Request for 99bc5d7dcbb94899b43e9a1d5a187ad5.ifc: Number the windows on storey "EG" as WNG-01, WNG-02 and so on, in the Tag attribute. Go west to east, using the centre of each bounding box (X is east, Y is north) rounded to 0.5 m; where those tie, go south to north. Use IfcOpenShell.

First a look at what the model holds.

```python
import ifcopenshell
import ifcopenshell.util.element
import ifcopenshell.util.placement

model = ifcopenshell.open("99bc5d7dcbb94899b43e9a1d5a187ad5.ifc")
print(model.schema)
storey = next(s for s in model.by_type("IfcBuildingStorey") if s.Name == "EG")
windows = [e for e in ifcopenshell.util.element.get_decomposition(storey) if e.is_a("IfcWindow")]
for e in sorted(windows, key=lambda e: e.id()):
    origin = ifcopenshell.util.placement.get_local_placement(e.ObjectPlacement)[:3, 3]
    print(e.id(), e.Tag, e.Name, origin.round(2) + 0.0, sep=" | ")
```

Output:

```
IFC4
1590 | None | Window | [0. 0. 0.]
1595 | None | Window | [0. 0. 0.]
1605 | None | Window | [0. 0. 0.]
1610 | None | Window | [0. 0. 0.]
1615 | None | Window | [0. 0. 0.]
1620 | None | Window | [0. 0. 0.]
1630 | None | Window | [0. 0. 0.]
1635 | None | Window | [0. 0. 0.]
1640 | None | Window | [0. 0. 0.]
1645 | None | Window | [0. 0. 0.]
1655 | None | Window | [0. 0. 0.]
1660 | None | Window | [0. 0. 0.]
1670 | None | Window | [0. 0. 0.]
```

```python
import ifcopenshell
import ifcopenshell.geom
import ifcopenshell.util.element
import ifcopenshell.util.shape

model = ifcopenshell.open("99bc5d7dcbb94899b43e9a1d5a187ad5.ifc")
settings = ifcopenshell.geom.settings()
settings.set("use-world-coords", True)


def centre(element):
    shape = ifcopenshell.geom.create_shape(settings, element)
    return ifcopenshell.util.shape.get_bbox_centroid(shape.geometry)


storey = next(s for s in model.by_type("IfcBuildingStorey") if s.Name == "EG")
windows = [e for e in ifcopenshell.util.element.get_decomposition(storey) if e.is_a("IfcWindow")]

# Insertion points can sit at a corner or the storey origin, so sort by the geometry (in metres).
centres = {e: centre(e) for e in windows}
windows.sort(key=lambda e: (round(centres[e][0] / 0.5), centres[e][1]))

for i, e in enumerate(windows, start=1):
    number = f"WNG-{i:02d}"
    e.Tag = number
    print(e.id(), number)

model.write("99bc5d7dcbb94899b43e9a1d5a187ad5_rev.ifc")
```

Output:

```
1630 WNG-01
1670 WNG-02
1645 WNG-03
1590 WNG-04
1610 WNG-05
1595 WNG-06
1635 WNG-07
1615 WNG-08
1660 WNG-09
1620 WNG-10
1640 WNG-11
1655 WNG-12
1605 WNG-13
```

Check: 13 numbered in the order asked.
